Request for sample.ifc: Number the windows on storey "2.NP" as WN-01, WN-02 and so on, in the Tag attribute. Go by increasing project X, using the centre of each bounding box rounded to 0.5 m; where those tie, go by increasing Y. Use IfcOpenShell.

First a look at what the model holds.

```python
import ifcopenshell
import ifcopenshell.util.element
import ifcopenshell.util.placement

model = ifcopenshell.open("sample.ifc")
print(model.schema)
storey = next(s for s in model.by_type("IfcBuildingStorey") if s.Name == "2.NP")
windows = [e for e in ifcopenshell.util.element.get_decomposition(storey) if e.is_a("IfcWindow")]
for e in sorted(windows, key=lambda e: e.id()):
    origin = ifcopenshell.util.placement.get_local_placement(e.ObjectPlacement)[:3, 3]
    print(e.id(), e.Tag, e.Name, origin.round(2) + 0.0, sep=" | ")
```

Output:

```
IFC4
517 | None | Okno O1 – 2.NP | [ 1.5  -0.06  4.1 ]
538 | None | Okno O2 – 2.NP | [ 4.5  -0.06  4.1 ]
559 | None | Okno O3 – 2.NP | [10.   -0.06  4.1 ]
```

```python
import ifcopenshell
import ifcopenshell.geom
import ifcopenshell.util.element
import ifcopenshell.util.shape

model = ifcopenshell.open("sample.ifc")
settings = ifcopenshell.geom.settings()
settings.set("use-world-coords", True)


def centre(element):
    shape = ifcopenshell.geom.create_shape(settings, element)
    return ifcopenshell.util.shape.get_bbox_centroid(shape.geometry)


storey = next(s for s in model.by_type("IfcBuildingStorey") if s.Name == "2.NP")
windows = [e for e in ifcopenshell.util.element.get_decomposition(storey) if e.is_a("IfcWindow")]

# Insertion points can sit at a corner or the storey origin, so sort by the geometry (in metres).
centres = {e: centre(e) for e in windows}
windows.sort(key=lambda e: (round(centres[e][0] / 0.5), centres[e][1]))

for i, e in enumerate(windows, start=1):
    number = f"WN-{i:02d}"
    e.Tag = number
    print(e.id(), number)

model.write("sample_updated.ifc")
```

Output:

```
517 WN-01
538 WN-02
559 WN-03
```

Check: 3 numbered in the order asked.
